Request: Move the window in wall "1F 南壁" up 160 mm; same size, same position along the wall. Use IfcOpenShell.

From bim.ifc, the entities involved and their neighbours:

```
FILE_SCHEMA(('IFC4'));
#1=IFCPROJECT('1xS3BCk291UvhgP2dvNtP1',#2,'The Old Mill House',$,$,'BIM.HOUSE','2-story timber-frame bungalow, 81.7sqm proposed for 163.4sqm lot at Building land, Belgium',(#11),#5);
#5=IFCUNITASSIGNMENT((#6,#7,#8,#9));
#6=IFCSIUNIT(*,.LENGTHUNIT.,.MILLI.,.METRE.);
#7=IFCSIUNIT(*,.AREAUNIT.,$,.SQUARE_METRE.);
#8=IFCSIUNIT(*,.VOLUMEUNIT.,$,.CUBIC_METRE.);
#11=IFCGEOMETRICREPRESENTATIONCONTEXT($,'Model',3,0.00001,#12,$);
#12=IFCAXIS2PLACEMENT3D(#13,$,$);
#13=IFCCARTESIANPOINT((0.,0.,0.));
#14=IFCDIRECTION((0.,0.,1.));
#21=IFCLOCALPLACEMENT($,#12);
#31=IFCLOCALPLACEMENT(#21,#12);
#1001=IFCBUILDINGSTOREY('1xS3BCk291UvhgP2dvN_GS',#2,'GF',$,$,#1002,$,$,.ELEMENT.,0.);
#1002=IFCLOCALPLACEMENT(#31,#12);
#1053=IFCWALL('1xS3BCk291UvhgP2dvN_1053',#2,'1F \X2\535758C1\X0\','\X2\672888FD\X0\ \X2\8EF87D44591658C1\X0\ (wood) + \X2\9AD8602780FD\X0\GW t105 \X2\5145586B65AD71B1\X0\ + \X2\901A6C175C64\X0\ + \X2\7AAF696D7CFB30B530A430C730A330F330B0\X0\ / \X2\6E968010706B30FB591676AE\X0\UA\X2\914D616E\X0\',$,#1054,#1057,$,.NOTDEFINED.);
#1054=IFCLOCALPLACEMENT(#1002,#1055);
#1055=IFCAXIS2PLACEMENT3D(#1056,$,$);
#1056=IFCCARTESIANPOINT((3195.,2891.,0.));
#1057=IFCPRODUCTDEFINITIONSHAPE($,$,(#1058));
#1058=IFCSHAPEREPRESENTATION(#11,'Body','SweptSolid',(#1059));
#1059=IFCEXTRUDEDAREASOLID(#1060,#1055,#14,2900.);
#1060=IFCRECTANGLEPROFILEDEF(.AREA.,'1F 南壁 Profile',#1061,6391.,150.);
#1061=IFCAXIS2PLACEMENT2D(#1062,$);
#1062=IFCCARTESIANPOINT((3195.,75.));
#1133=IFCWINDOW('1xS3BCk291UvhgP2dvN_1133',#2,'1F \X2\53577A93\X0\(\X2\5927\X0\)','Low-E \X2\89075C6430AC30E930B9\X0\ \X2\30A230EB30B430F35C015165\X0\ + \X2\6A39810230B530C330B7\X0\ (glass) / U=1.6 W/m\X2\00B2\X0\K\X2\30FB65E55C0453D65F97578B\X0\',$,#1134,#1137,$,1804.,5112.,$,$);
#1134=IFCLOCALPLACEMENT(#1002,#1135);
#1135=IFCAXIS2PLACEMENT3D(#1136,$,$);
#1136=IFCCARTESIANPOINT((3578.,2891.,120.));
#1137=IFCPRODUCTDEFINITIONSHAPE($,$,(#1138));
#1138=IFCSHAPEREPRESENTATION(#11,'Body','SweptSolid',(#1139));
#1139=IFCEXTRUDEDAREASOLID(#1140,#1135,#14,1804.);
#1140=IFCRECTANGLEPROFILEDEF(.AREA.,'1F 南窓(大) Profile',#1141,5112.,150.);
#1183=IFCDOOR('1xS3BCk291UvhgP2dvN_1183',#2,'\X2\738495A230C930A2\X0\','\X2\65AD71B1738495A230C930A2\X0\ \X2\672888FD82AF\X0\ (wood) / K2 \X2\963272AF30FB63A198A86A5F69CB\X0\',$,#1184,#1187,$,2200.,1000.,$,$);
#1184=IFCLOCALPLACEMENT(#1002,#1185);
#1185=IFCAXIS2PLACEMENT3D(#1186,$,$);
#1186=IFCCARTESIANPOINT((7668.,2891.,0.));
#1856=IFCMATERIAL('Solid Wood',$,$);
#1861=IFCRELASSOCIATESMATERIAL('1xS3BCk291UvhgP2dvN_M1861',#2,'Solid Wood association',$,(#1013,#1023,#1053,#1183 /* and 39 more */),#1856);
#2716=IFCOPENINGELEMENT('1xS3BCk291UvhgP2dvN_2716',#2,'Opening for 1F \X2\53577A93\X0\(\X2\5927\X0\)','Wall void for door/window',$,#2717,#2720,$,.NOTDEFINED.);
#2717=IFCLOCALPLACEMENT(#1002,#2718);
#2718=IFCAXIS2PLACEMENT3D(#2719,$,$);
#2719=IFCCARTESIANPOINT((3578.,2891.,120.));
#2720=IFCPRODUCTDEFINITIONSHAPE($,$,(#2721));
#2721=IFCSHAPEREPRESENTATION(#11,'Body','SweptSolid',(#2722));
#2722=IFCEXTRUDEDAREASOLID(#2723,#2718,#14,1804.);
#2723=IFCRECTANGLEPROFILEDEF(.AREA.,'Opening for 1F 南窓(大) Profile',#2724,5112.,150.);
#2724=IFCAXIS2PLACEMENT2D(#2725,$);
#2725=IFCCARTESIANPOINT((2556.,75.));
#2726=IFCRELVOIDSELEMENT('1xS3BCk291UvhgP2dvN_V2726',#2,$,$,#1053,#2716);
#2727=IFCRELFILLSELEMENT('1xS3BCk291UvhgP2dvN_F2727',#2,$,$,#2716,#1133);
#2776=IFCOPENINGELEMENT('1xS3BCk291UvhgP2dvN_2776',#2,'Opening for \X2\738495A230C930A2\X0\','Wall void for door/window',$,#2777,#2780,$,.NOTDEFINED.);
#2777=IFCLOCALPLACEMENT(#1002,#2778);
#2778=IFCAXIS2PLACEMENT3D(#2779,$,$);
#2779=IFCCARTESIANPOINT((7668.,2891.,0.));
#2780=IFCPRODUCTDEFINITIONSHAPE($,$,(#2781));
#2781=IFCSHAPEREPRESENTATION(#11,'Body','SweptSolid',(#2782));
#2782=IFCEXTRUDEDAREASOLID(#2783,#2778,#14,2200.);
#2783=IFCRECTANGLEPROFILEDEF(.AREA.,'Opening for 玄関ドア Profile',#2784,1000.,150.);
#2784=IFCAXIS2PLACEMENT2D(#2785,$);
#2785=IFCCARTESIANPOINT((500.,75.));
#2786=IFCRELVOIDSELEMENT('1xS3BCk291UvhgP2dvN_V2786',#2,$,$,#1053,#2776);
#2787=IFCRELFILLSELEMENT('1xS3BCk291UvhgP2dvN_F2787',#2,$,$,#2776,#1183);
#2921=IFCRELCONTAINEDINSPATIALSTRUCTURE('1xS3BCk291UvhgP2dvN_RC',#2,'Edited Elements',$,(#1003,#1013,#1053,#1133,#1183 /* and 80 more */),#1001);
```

```python
import numpy as np
import ifcopenshell
import ifcopenshell.api.geometry
import ifcopenshell.util.placement
import ifcopenshell.util.unit

model = ifcopenshell.open("bim.ifc")
unit_scale = ifcopenshell.util.unit.calculate_unit_scale(model)

window = model.by_guid("1xS3BCk291UvhgP2dvN_1133")
opening = window.FillsVoids[0].RelatingOpeningElement
dz = 0.16 / unit_scale

shift = np.array([0.0, 0.0, dz])
# The window is not placed relative to its opening, so move both.
for product in (opening, window):
    matrix = ifcopenshell.util.placement.get_local_placement(product.ObjectPlacement)
    matrix[:3, 3] += shift
    ifcopenshell.api.geometry.edit_object_placement(model, product=product, matrix=matrix, is_si=False)

print(f"moved by {dz * unit_scale:+.3f} m")

model.write("bim_v2.ifc")
```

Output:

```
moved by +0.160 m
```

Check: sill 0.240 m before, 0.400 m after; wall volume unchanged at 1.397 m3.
